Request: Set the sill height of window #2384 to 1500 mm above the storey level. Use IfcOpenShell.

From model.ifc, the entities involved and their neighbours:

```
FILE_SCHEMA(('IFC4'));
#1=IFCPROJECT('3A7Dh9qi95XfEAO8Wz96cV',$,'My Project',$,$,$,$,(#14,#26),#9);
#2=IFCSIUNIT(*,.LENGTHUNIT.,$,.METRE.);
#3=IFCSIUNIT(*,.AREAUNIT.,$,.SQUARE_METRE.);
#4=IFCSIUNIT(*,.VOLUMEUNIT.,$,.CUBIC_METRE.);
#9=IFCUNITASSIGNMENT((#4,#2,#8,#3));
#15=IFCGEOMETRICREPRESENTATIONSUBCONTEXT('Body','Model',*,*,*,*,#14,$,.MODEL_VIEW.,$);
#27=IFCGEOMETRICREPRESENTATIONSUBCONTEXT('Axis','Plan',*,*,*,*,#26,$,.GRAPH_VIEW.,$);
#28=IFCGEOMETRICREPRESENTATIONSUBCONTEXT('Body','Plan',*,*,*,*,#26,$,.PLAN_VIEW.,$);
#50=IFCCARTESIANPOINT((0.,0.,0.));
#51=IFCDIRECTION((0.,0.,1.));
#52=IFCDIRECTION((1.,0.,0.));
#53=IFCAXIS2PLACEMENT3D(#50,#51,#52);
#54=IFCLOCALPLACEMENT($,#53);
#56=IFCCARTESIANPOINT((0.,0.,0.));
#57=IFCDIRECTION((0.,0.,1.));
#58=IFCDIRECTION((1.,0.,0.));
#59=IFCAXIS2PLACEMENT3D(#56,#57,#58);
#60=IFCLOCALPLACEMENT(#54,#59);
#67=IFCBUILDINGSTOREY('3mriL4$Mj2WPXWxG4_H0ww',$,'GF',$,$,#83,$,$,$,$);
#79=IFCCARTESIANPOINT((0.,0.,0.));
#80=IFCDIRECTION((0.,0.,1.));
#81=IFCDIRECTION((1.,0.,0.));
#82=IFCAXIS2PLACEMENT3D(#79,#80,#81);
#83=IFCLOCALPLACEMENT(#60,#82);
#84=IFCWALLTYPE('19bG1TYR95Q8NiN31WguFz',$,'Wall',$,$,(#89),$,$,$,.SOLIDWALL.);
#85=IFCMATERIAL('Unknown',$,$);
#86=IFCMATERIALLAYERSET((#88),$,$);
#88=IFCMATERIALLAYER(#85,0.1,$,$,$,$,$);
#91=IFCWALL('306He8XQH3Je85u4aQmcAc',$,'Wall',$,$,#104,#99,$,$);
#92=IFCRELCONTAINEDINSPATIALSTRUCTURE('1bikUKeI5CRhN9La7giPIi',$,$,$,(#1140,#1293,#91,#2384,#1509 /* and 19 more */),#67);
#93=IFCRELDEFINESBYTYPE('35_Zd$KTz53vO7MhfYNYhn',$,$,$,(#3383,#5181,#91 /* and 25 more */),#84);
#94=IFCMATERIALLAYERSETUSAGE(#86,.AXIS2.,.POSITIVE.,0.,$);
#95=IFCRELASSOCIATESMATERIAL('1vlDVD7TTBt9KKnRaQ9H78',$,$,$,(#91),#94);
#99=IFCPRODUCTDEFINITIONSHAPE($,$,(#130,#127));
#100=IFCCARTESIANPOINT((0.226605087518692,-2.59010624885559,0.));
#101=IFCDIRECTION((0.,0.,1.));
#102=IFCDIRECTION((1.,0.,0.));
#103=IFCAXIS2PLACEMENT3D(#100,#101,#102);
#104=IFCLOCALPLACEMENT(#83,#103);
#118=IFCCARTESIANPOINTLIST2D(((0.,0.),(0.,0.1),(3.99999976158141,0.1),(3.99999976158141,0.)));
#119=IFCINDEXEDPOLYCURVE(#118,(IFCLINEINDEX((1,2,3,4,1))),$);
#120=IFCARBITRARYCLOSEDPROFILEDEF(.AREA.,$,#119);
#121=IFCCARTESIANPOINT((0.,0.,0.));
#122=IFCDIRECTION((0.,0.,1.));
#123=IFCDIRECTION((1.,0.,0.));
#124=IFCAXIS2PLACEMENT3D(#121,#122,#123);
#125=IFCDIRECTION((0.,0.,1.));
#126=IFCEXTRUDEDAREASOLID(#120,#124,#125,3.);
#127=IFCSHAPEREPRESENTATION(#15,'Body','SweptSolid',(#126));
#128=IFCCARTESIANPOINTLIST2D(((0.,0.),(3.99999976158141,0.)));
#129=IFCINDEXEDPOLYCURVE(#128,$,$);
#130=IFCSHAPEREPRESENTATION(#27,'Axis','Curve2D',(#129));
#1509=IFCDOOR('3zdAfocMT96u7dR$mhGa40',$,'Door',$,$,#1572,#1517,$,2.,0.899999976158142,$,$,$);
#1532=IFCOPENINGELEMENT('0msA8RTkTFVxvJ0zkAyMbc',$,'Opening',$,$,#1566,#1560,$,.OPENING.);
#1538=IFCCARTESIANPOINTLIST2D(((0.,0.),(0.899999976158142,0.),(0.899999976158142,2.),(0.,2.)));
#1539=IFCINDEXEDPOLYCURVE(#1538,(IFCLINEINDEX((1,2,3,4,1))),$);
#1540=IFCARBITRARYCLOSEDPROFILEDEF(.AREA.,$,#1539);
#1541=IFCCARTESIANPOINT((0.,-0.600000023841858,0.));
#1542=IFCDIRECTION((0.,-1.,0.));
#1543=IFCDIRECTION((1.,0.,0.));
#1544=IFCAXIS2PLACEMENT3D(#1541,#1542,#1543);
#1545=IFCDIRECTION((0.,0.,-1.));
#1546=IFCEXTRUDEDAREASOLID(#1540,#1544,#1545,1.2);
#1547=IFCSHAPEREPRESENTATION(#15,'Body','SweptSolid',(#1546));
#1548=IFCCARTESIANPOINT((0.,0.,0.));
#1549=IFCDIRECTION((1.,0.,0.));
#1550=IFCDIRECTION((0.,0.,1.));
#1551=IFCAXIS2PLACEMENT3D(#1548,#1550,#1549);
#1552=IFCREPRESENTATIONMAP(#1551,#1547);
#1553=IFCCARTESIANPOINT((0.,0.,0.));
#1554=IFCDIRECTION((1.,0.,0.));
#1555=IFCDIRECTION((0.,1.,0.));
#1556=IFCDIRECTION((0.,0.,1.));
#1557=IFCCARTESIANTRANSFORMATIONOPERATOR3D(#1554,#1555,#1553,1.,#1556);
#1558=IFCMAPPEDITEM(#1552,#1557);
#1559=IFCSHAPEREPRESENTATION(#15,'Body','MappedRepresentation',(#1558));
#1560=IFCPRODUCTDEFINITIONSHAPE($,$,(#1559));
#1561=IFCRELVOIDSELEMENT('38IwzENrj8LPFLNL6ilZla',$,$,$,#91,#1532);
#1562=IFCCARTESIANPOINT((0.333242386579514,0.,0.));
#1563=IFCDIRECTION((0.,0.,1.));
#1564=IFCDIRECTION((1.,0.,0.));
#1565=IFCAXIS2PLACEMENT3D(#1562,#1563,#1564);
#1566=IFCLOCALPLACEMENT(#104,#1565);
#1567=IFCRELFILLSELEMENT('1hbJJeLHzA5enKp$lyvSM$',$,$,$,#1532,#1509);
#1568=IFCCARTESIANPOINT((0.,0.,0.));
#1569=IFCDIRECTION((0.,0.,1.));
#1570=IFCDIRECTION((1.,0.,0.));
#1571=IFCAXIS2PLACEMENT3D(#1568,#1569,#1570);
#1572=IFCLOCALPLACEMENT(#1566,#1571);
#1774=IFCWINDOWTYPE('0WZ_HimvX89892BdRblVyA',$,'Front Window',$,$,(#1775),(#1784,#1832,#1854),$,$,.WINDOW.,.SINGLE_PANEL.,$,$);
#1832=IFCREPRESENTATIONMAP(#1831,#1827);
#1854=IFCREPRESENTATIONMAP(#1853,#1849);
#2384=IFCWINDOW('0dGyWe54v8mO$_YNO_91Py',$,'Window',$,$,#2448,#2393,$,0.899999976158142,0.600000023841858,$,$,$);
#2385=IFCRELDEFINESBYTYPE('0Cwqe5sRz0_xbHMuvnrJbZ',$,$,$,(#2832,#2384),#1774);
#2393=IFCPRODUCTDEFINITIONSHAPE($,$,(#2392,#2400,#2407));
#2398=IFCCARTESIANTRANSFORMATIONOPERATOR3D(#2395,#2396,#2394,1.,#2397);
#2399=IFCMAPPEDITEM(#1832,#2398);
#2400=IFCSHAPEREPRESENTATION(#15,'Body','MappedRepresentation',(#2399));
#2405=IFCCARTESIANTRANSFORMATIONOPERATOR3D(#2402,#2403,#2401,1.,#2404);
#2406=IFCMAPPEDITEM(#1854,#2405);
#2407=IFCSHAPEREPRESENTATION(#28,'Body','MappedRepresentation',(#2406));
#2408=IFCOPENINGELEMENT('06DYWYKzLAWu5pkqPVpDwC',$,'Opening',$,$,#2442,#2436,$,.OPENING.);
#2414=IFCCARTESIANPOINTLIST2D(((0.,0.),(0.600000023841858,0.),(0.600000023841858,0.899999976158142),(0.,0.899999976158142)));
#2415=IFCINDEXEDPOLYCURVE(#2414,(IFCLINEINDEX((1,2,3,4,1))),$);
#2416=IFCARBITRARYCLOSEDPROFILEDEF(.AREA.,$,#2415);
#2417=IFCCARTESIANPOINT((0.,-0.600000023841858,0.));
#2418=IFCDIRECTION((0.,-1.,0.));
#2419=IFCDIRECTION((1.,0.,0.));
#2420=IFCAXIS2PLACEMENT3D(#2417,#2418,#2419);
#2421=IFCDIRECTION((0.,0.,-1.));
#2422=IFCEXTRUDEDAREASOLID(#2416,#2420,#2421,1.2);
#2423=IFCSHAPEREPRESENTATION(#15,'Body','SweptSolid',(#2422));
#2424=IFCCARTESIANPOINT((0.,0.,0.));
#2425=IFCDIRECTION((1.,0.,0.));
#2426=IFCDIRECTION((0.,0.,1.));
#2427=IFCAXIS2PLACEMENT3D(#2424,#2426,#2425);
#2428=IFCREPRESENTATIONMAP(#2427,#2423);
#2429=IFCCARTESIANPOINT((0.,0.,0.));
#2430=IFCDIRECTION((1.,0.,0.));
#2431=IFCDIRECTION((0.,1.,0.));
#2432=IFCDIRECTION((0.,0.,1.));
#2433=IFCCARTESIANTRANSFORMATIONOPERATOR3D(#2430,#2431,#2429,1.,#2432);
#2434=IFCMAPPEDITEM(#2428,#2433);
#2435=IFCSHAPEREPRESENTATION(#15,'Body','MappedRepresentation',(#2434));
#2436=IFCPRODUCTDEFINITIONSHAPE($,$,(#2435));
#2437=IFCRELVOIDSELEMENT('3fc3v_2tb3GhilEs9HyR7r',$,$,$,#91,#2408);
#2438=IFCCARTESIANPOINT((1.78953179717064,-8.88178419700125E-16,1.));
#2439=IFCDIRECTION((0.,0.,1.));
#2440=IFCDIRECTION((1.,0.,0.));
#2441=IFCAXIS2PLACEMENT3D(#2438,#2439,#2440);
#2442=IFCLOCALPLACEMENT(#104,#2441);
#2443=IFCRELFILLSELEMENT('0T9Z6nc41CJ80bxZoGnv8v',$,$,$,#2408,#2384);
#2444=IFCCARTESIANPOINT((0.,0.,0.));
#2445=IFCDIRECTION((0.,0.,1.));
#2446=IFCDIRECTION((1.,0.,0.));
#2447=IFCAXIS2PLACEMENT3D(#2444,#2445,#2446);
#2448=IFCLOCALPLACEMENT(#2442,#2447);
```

```python
import numpy as np
import ifcopenshell
import ifcopenshell.api.geometry
import ifcopenshell.geom
import ifcopenshell.util.element
import ifcopenshell.util.placement
import ifcopenshell.util.shape
import ifcopenshell.util.unit

model = ifcopenshell.open("model.ifc")
unit_scale = ifcopenshell.util.unit.calculate_unit_scale(model)

window = model.by_guid("0dGyWe54v8mO$_YNO_91Py")
opening = window.FillsVoids[0].RelatingOpeningElement
storey = ifcopenshell.util.element.get_container(window, ifc_class="IfcBuildingStorey")
level = ifcopenshell.util.placement.get_local_placement(storey.ObjectPlacement)[2, 3]

# The opening's origin need not be at the sill, so measure its lowest point.
shape = ifcopenshell.geom.create_shape(ifcopenshell.geom.settings(), opening)
bottom = ifcopenshell.util.shape.get_shape_bottom_elevation(shape, shape.geometry) / unit_scale
dz = level + 1.5 - bottom

shift = np.array([0.0, 0.0, dz])
# The window is placed relative to its opening, so it follows when the opening moves.
matrix = ifcopenshell.util.placement.get_local_placement(opening.ObjectPlacement)
matrix[:3, 3] += shift
ifcopenshell.api.geometry.edit_object_placement(
    model, product=opening, matrix=matrix, is_si=False, should_transform_children=True
)

print(f"moved by {dz * unit_scale:+.3f} m")

model.write("model_edited.ifc")
```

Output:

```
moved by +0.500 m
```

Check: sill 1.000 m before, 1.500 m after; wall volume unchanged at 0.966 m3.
